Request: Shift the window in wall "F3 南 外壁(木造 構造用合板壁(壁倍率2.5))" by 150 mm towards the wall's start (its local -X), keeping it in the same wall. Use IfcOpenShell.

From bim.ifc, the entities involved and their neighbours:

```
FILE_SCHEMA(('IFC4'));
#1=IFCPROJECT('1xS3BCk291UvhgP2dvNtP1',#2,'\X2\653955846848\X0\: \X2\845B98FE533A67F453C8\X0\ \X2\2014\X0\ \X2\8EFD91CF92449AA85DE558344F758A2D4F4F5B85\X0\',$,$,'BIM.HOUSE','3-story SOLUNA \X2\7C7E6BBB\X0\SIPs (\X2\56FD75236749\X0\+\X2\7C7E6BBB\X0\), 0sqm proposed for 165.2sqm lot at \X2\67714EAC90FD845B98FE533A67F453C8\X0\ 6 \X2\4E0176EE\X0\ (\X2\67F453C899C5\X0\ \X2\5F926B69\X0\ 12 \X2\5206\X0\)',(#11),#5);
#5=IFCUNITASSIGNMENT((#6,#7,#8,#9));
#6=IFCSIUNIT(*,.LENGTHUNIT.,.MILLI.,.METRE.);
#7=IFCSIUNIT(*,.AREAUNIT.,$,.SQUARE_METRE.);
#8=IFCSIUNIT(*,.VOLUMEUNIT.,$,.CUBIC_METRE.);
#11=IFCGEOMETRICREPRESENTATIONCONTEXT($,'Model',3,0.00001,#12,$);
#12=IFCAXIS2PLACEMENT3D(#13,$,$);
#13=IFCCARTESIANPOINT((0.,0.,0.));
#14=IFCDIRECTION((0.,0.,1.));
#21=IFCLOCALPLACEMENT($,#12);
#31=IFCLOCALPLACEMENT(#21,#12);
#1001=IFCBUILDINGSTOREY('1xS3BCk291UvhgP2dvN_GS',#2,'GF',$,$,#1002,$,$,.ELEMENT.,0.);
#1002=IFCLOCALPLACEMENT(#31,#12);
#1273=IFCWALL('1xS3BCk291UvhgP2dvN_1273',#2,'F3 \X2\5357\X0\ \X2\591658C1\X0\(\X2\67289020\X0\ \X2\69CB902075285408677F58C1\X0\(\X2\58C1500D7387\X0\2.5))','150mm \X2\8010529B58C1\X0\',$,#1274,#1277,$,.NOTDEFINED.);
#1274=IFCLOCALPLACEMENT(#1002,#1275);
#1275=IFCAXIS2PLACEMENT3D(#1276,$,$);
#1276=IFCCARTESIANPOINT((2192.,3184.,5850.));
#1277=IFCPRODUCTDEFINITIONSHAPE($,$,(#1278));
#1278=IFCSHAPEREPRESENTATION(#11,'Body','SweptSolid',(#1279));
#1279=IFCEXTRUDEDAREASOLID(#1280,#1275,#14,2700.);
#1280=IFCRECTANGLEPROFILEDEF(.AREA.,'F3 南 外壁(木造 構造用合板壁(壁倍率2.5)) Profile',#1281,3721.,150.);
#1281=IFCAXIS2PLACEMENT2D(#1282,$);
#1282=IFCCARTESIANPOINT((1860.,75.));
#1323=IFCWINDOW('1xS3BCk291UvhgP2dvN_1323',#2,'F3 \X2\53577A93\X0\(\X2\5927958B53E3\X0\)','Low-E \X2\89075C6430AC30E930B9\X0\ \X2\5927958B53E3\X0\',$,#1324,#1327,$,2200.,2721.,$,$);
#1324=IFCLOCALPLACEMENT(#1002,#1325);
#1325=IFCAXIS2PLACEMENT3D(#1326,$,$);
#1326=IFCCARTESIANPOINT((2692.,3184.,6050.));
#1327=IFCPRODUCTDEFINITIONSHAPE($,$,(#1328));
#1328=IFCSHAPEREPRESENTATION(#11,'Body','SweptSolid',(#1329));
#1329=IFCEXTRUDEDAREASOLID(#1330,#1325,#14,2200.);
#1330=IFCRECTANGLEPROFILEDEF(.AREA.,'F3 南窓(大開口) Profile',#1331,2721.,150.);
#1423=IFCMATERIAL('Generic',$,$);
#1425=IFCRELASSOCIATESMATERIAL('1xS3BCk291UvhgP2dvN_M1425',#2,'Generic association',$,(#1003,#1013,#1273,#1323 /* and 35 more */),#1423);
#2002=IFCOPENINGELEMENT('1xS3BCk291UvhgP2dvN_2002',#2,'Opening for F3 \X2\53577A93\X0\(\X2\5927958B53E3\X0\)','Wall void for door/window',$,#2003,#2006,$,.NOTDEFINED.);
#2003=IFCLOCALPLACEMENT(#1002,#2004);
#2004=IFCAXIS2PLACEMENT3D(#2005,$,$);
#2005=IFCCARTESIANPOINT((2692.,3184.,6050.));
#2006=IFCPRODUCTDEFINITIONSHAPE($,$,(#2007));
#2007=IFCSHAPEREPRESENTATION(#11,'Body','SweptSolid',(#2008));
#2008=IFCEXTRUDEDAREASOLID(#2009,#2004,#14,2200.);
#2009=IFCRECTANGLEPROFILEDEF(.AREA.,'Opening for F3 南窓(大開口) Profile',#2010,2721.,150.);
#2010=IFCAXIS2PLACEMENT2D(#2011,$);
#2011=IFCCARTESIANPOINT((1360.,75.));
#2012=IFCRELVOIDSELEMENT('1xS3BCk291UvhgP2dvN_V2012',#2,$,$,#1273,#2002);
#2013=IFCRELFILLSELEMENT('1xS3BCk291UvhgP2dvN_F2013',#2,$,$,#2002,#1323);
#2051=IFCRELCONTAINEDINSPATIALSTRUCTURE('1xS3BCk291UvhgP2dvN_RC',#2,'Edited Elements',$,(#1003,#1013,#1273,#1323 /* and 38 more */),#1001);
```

```python
import ifcopenshell
import ifcopenshell.api.geometry
import ifcopenshell.util.placement
import ifcopenshell.util.unit

model = ifcopenshell.open("bim.ifc")
unit_scale = ifcopenshell.util.unit.calculate_unit_scale(model)

window = model.by_guid("1xS3BCk291UvhgP2dvN_1323")
opening = window.FillsVoids[0].RelatingOpeningElement
wall = opening.VoidsElements[0].RelatingBuildingElement

wall_matrix = ifcopenshell.util.placement.get_local_placement(wall.ObjectPlacement)
shift = wall_matrix[:3, 0] * -0.15 / unit_scale
before = ifcopenshell.util.placement.get_local_placement(window.ObjectPlacement)[:3, 3].copy()

# The window is not placed relative to its opening, so move both.
for product in (opening, window):
    matrix = ifcopenshell.util.placement.get_local_placement(product.ObjectPlacement)
    matrix[:3, 3] += shift
    ifcopenshell.api.geometry.edit_object_placement(model, product=product, matrix=matrix, is_si=False)

after = ifcopenshell.util.placement.get_local_placement(window.ObjectPlacement)[:3, 3]
print("window moved by", (after - before).round(3) + 0.0)

model.write("bim-out.ifc")
```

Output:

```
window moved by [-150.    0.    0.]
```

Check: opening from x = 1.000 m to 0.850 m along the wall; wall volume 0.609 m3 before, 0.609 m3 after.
